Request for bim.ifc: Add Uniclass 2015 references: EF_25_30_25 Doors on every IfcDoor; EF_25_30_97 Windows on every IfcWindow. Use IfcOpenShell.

First a look at what the model holds.

```python
import ifcopenshell

model = ifcopenshell.open("bim.ifc")
print(model.schema)
print("classifications:", [c.Name for c in model.by_type("IfcClassification")])
for ifc_class in ("IfcDoor", "IfcRoof", "IfcStair", "IfcWall", "IfcWindow"):
    print(ifc_class, len(model.by_type(ifc_class)))
```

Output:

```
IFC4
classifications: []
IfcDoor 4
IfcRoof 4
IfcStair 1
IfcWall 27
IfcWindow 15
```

```python
import ifcopenshell
import ifcopenshell.api.classification

model = ifcopenshell.open("bim.ifc")

system = ifcopenshell.api.classification.add_classification(model, classification="Uniclass 2015")

codes = {
    "IfcDoor": ("EF_25_30_25", "Doors"),
    "IfcWindow": ("EF_25_30_97", "Windows"),
}
for ifc_class, (code, name) in codes.items():
    products = model.by_type(ifc_class)
    ifcopenshell.api.classification.add_reference(
        model, products=products, classification=system, identification=code, name=name
    )
    print(code, len(products))

model.write("bim_updated.ifc")
```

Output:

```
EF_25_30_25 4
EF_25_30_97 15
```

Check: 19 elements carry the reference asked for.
